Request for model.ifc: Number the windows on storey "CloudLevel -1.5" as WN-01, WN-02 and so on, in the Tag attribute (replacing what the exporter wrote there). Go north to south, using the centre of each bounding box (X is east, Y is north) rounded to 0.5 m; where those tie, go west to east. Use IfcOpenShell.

First a look at what the model holds.

```python
import ifcopenshell
import ifcopenshell.util.element
import ifcopenshell.util.placement

model = ifcopenshell.open("model.ifc")
print(model.schema)
storey = next(s for s in model.by_type("IfcBuildingStorey") if s.Name == "CloudLevel -1.5")
windows = [e for e in ifcopenshell.util.element.get_decomposition(storey) if e.is_a("IfcWindow")]
for e in sorted(windows, key=lambda e: e.id()):
    origin = ifcopenshell.util.placement.get_local_placement(e.ObjectPlacement)[:3, 3]
    print(e.id(), e.Tag, e.Name, origin.round(2) + 0.0, sep=" | ")
```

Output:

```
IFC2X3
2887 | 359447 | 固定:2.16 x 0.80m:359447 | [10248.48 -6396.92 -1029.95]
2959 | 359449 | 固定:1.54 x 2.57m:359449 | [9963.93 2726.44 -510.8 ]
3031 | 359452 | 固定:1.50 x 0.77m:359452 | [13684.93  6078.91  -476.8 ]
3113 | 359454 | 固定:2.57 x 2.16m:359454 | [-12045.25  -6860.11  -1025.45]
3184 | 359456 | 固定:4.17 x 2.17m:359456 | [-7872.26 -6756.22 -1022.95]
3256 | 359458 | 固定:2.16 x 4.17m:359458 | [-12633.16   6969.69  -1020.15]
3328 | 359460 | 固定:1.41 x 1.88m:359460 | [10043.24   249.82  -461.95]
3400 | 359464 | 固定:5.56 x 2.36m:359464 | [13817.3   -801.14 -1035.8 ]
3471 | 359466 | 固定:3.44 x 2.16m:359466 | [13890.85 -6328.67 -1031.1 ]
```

```python
import ifcopenshell
import ifcopenshell.geom
import ifcopenshell.util.element
import ifcopenshell.util.shape

model = ifcopenshell.open("model.ifc")
settings = ifcopenshell.geom.settings()
settings.set("use-world-coords", True)


def centre(element):
    shape = ifcopenshell.geom.create_shape(settings, element)
    return ifcopenshell.util.shape.get_bbox_centroid(shape.geometry)


storey = next(s for s in model.by_type("IfcBuildingStorey") if s.Name == "CloudLevel -1.5")
windows = [e for e in ifcopenshell.util.element.get_decomposition(storey) if e.is_a("IfcWindow")]

# Insertion points can sit at a corner or the storey origin, so sort by the geometry (in metres).
centres = {e: centre(e) for e in windows}
windows.sort(key=lambda e: (-round(centres[e][1] / 0.5), centres[e][0]))

for i, e in enumerate(windows, start=1):
    number = f"WN-{i:02d}"
    e.Tag = number
    print(e.id(), number)

model.write("model-out.ifc")
```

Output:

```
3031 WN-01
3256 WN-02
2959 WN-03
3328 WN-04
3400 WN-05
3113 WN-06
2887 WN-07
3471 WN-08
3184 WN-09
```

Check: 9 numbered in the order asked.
